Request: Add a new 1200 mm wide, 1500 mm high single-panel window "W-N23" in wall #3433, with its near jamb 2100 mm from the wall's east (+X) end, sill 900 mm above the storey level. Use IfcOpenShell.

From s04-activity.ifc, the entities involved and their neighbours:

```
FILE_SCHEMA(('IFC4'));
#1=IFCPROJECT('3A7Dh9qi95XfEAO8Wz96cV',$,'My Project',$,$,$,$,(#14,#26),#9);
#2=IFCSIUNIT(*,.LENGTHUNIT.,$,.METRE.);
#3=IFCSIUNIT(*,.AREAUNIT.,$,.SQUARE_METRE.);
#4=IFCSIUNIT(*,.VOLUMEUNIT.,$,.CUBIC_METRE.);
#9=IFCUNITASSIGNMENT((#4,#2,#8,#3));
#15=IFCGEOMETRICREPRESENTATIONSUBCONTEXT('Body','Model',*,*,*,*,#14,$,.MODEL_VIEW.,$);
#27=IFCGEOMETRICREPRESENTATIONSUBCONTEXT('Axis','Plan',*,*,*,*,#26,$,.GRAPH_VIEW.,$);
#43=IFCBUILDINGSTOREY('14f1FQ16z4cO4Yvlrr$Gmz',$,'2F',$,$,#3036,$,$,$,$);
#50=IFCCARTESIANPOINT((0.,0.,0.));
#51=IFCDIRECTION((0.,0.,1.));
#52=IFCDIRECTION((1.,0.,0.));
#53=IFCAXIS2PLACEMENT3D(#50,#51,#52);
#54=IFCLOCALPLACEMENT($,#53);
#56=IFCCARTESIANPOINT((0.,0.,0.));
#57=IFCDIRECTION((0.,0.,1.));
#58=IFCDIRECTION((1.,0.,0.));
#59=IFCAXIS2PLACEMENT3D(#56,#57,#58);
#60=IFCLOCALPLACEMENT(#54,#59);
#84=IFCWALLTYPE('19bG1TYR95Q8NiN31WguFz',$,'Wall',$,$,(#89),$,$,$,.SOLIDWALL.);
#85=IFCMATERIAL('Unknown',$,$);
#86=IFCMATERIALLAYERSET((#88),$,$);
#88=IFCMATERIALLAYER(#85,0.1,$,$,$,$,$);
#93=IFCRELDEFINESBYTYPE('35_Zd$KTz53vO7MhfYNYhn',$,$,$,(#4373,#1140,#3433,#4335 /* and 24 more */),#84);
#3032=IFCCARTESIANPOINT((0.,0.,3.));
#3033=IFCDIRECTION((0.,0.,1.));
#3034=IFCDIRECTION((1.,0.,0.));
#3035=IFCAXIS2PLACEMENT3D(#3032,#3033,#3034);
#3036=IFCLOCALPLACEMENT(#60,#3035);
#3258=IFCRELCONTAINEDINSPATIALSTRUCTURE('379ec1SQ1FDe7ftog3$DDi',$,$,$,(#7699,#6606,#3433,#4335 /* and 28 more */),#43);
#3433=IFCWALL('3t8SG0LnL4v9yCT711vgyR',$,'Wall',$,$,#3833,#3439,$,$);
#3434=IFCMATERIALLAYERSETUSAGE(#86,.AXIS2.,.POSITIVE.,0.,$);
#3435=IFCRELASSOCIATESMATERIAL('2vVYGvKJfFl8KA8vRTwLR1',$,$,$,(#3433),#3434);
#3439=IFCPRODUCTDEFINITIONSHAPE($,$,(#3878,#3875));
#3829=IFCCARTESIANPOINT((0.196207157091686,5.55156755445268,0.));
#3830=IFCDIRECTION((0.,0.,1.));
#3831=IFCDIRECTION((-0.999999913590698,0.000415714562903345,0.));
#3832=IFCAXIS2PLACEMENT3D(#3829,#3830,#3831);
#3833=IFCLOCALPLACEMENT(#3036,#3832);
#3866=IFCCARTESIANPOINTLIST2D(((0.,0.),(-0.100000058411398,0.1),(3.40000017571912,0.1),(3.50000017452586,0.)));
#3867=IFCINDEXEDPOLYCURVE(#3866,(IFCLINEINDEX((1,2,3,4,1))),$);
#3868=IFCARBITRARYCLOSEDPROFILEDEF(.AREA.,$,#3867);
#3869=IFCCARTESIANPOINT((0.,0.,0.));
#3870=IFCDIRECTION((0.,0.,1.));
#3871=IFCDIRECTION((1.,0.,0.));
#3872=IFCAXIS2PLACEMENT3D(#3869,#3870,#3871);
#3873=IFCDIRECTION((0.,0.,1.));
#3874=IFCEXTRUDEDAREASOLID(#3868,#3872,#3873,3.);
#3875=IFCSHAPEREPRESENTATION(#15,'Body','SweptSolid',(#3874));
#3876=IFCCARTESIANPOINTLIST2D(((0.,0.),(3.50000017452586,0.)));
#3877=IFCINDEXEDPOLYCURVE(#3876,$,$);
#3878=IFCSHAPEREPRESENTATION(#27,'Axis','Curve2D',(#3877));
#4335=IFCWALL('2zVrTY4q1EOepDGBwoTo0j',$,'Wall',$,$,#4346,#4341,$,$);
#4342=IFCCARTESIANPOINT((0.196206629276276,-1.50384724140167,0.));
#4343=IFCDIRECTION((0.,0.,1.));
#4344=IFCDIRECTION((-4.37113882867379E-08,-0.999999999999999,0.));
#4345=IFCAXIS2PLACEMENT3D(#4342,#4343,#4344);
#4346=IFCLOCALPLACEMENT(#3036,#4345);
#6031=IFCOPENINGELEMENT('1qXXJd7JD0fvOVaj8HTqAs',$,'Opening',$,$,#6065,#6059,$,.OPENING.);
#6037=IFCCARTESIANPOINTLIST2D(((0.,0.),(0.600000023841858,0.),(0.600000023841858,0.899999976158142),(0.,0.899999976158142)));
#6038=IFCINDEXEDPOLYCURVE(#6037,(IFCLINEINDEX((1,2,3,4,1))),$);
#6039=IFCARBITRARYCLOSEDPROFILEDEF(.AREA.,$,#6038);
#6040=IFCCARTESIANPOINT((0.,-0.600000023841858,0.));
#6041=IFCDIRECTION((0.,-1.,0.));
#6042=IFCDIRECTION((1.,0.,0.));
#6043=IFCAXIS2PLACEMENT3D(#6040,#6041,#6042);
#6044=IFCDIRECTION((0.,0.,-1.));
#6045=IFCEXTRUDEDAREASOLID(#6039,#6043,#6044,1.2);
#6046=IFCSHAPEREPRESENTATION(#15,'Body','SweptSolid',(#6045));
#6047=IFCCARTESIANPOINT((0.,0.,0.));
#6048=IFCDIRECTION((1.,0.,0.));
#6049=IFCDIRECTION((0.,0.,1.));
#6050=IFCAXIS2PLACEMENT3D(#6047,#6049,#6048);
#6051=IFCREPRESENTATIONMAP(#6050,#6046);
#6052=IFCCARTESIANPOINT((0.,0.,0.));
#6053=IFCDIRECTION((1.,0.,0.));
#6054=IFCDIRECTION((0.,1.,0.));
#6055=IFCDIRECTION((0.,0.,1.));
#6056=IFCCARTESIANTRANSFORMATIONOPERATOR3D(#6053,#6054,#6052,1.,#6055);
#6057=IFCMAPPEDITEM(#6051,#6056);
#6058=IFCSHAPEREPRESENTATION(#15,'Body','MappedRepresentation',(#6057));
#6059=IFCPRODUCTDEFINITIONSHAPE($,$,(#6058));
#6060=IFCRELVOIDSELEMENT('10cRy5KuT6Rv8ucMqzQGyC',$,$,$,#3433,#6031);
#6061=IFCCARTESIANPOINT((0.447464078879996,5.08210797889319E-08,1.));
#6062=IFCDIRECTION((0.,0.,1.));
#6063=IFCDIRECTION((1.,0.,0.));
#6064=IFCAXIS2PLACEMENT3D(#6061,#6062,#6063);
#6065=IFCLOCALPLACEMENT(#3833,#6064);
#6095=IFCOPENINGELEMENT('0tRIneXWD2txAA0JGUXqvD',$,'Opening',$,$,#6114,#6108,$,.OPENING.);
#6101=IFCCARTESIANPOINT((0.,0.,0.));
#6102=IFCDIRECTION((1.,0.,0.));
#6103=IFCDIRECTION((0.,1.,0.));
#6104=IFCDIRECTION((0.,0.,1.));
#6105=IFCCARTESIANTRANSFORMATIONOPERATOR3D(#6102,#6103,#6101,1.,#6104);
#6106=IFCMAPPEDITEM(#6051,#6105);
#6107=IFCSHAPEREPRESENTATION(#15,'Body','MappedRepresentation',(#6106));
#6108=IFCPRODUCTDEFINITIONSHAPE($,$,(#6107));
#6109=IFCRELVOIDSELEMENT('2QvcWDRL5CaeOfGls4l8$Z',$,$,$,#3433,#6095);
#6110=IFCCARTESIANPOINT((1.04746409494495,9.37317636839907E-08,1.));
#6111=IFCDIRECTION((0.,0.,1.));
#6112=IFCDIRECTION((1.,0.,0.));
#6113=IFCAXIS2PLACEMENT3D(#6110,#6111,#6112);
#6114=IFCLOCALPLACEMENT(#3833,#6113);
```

```python
import numpy as np
import ifcopenshell
import ifcopenshell.api.feature
import ifcopenshell.api.geometry
import ifcopenshell.api.root
import ifcopenshell.api.spatial
import ifcopenshell.geom
import ifcopenshell.util.element
import ifcopenshell.util.placement
import ifcopenshell.util.representation
import ifcopenshell.util.shape
import ifcopenshell.util.unit

model = ifcopenshell.open("s04-activity.ifc")
unit_scale = ifcopenshell.util.unit.calculate_unit_scale(model)
settings = ifcopenshell.geom.settings()


def volume(element):
    """Net volume in cubic metres, openings subtracted."""
    shape = ifcopenshell.geom.create_shape(settings, element)
    return ifcopenshell.util.shape.get_volume(shape.geometry)


wall = model.by_guid("3t8SG0LnL4v9yCT711vgyR")
storey = ifcopenshell.util.element.get_container(wall, ifc_class="IfcBuildingStorey")
context = ifcopenshell.util.representation.get_context(model, "Model", "Body", "MODEL_VIEW")
before = volume(wall)

width, height, from_end, sill = 1.2, 1.5, 2.1, 0.9  # metres

# The wall runs along its own X axis, and the end named is its -X end.
wall_shape = ifcopenshell.geom.create_shape(settings, wall)
x, y, z = ifcopenshell.util.shape.get_vertices(wall_shape.geometry).T
start = x.min() + from_end
face, thickness = float(y.min()), float(y.max() - y.min())
wall_matrix = ifcopenshell.util.placement.get_local_placement(wall.ObjectPlacement)
level = ifcopenshell.util.placement.get_local_placement(storey.ObjectPlacement)[2, 3]


def in_wall(x, y):
    """Placement at x, y metres in the wall's axes, at sill height."""
    matrix = wall_matrix.copy()
    matrix[:, 3] = wall_matrix @ np.array([x / unit_scale, y / unit_scale, 0.0, 1.0])
    matrix[2, 3] = level + sill / unit_scale
    return matrix


# Opening: a box that overshoots both wall faces by 50 mm.
opening = ifcopenshell.api.root.create_entity(model, ifc_class="IfcOpeningElement", predefined_type="OPENING")
box = ifcopenshell.api.geometry.add_wall_representation(
    model, context=context, length=width, height=height, thickness=thickness + 0.1
)
ifcopenshell.api.geometry.assign_representation(model, product=opening, representation=box)
ifcopenshell.api.geometry.edit_object_placement(model, product=opening, matrix=in_wall(start, face - 0.05), is_si=False)
ifcopenshell.api.feature.add_feature(model, feature=opening, element=wall)

window = ifcopenshell.api.root.create_entity(model, ifc_class="IfcWindow", name="W-N23", predefined_type="WINDOW")
window.OverallWidth, window.OverallHeight = width / unit_scale, height / unit_scale
window.PartitioningType = "SINGLE_PANEL"
body = ifcopenshell.api.geometry.add_window_representation(
    model,
    context=context,
    overall_width=window.OverallWidth,
    overall_height=window.OverallHeight,
    partition_type="SINGLE_PANEL",
)
ifcopenshell.api.geometry.assign_representation(model, product=window, representation=body)
ifcopenshell.api.spatial.assign_container(model, products=[window], relating_structure=storey)
ifcopenshell.api.feature.add_filling(model, opening=opening, element=window)

# Centre the window in the wall's thickness.
ifcopenshell.api.geometry.edit_object_placement(model, product=window, matrix=in_wall(start, face), is_si=False)
window_shape = ifcopenshell.geom.create_shape(settings, window)
depth = ifcopenshell.util.shape.get_vertices(window_shape.geometry)[:, 1]
offset = face + thickness / 2 - (depth.min() + depth.max()) / 2
ifcopenshell.api.geometry.edit_object_placement(model, product=window, matrix=in_wall(start, offset), is_si=False)

after = volume(wall)

print(f"wall volume {before:.3f} -> {after:.3f} m3")

model.write("s04-activity_updated.ifc")
```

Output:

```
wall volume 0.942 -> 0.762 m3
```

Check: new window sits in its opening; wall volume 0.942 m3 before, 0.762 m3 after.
